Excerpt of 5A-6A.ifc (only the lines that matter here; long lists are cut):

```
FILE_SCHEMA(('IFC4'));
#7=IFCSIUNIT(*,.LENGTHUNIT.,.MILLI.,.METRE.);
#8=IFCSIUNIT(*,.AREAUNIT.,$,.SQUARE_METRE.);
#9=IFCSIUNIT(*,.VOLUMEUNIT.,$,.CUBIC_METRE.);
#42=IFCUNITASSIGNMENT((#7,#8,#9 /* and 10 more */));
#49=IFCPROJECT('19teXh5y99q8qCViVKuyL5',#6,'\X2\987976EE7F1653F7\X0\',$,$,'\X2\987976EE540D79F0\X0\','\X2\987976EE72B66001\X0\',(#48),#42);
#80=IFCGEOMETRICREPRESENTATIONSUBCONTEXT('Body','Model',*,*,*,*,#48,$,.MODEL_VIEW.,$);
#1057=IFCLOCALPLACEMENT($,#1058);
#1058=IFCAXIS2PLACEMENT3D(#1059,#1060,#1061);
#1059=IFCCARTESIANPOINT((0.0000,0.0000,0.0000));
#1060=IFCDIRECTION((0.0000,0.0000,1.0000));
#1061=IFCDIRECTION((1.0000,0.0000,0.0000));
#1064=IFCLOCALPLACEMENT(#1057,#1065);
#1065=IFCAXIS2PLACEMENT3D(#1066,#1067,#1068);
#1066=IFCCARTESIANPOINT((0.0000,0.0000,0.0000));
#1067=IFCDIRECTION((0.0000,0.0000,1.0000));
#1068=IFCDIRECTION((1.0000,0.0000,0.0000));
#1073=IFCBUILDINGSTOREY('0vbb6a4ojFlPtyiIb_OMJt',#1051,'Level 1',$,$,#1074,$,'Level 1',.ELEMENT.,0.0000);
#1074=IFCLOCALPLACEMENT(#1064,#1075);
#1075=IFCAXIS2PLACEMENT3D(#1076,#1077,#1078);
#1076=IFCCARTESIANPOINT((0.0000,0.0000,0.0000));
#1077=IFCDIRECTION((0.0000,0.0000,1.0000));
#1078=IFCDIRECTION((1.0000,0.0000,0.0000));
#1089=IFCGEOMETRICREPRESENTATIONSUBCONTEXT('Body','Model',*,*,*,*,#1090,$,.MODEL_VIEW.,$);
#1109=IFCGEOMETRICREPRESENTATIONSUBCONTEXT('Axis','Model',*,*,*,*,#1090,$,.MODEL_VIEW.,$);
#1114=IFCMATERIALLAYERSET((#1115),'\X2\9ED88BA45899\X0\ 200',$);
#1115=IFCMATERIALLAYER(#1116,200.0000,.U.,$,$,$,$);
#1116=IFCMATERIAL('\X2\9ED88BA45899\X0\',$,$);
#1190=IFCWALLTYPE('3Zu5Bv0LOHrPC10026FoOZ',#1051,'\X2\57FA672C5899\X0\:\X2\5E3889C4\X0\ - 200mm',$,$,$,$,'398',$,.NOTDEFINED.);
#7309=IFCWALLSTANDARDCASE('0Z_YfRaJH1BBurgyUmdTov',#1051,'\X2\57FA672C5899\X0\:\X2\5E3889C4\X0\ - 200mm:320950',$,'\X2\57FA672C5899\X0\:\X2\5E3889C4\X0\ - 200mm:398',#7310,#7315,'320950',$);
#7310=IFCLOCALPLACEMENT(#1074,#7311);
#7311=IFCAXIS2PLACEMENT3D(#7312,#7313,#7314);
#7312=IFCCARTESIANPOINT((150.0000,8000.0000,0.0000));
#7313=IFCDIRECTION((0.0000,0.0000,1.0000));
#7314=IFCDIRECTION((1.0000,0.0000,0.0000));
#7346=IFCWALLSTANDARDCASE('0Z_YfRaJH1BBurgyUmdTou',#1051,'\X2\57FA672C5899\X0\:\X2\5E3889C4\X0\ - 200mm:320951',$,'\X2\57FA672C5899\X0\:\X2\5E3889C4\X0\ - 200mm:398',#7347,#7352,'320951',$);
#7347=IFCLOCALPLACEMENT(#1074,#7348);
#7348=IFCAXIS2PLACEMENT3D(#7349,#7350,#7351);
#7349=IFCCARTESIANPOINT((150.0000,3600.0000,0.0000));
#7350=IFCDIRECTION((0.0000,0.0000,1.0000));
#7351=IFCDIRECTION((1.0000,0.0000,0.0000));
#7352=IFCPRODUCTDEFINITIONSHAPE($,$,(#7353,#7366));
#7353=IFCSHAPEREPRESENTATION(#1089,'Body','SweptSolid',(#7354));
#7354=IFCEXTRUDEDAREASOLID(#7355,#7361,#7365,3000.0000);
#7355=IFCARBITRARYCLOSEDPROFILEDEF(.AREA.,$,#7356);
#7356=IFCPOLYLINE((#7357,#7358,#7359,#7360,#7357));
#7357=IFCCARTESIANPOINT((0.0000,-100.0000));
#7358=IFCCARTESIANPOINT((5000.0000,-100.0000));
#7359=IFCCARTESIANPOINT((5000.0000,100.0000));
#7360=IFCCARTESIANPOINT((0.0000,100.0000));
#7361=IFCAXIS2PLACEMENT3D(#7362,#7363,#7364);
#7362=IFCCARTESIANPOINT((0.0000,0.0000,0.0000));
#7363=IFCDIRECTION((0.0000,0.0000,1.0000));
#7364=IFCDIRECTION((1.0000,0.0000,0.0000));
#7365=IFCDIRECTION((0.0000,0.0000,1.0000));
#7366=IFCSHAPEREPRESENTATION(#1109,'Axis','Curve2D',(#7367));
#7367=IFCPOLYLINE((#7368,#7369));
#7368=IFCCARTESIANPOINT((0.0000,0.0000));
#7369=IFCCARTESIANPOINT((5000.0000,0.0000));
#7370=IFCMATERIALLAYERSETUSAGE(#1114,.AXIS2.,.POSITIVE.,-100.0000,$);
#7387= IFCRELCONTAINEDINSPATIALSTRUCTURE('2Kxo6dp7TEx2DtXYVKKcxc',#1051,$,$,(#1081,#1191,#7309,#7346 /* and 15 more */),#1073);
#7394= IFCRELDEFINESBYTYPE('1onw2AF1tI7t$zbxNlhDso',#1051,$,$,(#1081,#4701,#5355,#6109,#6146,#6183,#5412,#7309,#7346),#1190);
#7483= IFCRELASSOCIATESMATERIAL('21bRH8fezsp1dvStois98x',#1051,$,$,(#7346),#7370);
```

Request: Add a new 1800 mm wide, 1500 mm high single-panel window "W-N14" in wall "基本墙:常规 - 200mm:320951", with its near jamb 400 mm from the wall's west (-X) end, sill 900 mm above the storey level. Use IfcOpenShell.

```python
import numpy as np
import ifcopenshell
import ifcopenshell.api.feature
import ifcopenshell.api.geometry
import ifcopenshell.api.root
import ifcopenshell.api.spatial
import ifcopenshell.geom
import ifcopenshell.util.element
import ifcopenshell.util.placement
import ifcopenshell.util.representation
import ifcopenshell.util.shape
import ifcopenshell.util.unit

model = ifcopenshell.open("5A-6A.ifc")
unit_scale = ifcopenshell.util.unit.calculate_unit_scale(model)
settings = ifcopenshell.geom.settings()


def volume(element):
    """Net volume in cubic metres, openings subtracted."""
    shape = ifcopenshell.geom.create_shape(settings, element)
    return ifcopenshell.util.shape.get_volume(shape.geometry)


wall = model.by_id(7346)
storey = ifcopenshell.util.element.get_container(wall, ifc_class="IfcBuildingStorey")
context = ifcopenshell.util.representation.get_context(model, "Model", "Body", "MODEL_VIEW")
before = volume(wall)

width, height, from_end, sill = 1.8, 1.5, 0.4, 0.9  # metres

# The wall runs along its own X axis, and the end named is its -X end.
wall_shape = ifcopenshell.geom.create_shape(settings, wall)
x, y, z = ifcopenshell.util.shape.get_vertices(wall_shape.geometry).T
start = x.min() + from_end
face, thickness = float(y.min()), float(y.max() - y.min())
wall_matrix = ifcopenshell.util.placement.get_local_placement(wall.ObjectPlacement)
level = ifcopenshell.util.placement.get_local_placement(storey.ObjectPlacement)[2, 3]


def in_wall(x, y):
    """Placement at x, y metres in the wall's axes, at sill height."""
    matrix = wall_matrix.copy()
    matrix[:, 3] = wall_matrix @ np.array([x / unit_scale, y / unit_scale, 0.0, 1.0])
    matrix[2, 3] = level + sill / unit_scale
    return matrix


# Opening: a box that overshoots both wall faces by 50 mm.
opening = ifcopenshell.api.root.create_entity(model, ifc_class="IfcOpeningElement", predefined_type="OPENING")
box = ifcopenshell.api.geometry.add_wall_representation(
    model, context=context, length=width, height=height, thickness=thickness + 0.1
)
ifcopenshell.api.geometry.assign_representation(model, product=opening, representation=box)
ifcopenshell.api.geometry.edit_object_placement(model, product=opening, matrix=in_wall(start, face - 0.05), is_si=False)
ifcopenshell.api.feature.add_feature(model, feature=opening, element=wall)

window = ifcopenshell.api.root.create_entity(model, ifc_class="IfcWindow", name="W-N14", predefined_type="WINDOW")
window.OverallWidth, window.OverallHeight = width / unit_scale, height / unit_scale
window.PartitioningType = "SINGLE_PANEL"
body = ifcopenshell.api.geometry.add_window_representation(
    model,
    context=context,
    overall_width=window.OverallWidth,
    overall_height=window.OverallHeight,
    partition_type="SINGLE_PANEL",
)
ifcopenshell.api.geometry.assign_representation(model, product=window, representation=body)
ifcopenshell.api.spatial.assign_container(model, products=[window], relating_structure=storey)
ifcopenshell.api.feature.add_filling(model, opening=opening, element=window)

# Centre the window in the wall's thickness.
ifcopenshell.api.geometry.edit_object_placement(model, product=window, matrix=in_wall(start, face), is_si=False)
window_shape = ifcopenshell.geom.create_shape(settings, window)
depth = ifcopenshell.util.shape.get_vertices(window_shape.geometry)[:, 1]
offset = face + thickness / 2 - (depth.min() + depth.max()) / 2
ifcopenshell.api.geometry.edit_object_placement(model, product=window, matrix=in_wall(start, offset), is_si=False)

after = volume(wall)

print(f"wall volume {before:.3f} -> {after:.3f} m3")

model.write("5A-6A_edited.ifc")
```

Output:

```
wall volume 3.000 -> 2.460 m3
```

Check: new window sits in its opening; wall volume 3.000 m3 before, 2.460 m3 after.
